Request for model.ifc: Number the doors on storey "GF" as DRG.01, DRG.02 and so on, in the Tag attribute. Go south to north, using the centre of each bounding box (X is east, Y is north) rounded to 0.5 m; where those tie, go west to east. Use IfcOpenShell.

First a look at what the model holds.

```python
import ifcopenshell
import ifcopenshell.util.element
import ifcopenshell.util.placement

model = ifcopenshell.open("model.ifc")
print(model.schema)
storey = next(s for s in model.by_type("IfcBuildingStorey") if s.Name == "GF")
doors = [e for e in ifcopenshell.util.element.get_decomposition(storey) if e.is_a("IfcDoor")]
for e in sorted(doors, key=lambda e: e.id()):
    origin = ifcopenshell.util.placement.get_local_placement(e.ObjectPlacement)[:3, 3]
    print(e.id(), e.Tag, e.Name, origin.round(2) + 0.0, sep=" | ")
```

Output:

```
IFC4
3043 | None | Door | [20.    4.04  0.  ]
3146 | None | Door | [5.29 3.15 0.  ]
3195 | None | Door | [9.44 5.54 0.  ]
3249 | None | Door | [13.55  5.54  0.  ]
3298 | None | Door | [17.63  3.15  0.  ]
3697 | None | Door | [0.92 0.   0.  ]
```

```python
import ifcopenshell
import ifcopenshell.geom
import ifcopenshell.util.element
import ifcopenshell.util.shape

model = ifcopenshell.open("model.ifc")
settings = ifcopenshell.geom.settings()
settings.set("use-world-coords", True)


def centre(element):
    shape = ifcopenshell.geom.create_shape(settings, element)
    return ifcopenshell.util.shape.get_bbox_centroid(shape.geometry)


storey = next(s for s in model.by_type("IfcBuildingStorey") if s.Name == "GF")
doors = [e for e in ifcopenshell.util.element.get_decomposition(storey) if e.is_a("IfcDoor")]

# Insertion points can sit at a corner or the storey origin, so sort by the geometry (in metres).
centres = {e: centre(e) for e in doors}
doors.sort(key=lambda e: (round(centres[e][1] / 0.5), centres[e][0]))

for i, e in enumerate(doors, start=1):
    number = f"DRG.{i:02d}"
    e.Tag = number
    print(e.id(), number)

model.write("model-out.ifc")
```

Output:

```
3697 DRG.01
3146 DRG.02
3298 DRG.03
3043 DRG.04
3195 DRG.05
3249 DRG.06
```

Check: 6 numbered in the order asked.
